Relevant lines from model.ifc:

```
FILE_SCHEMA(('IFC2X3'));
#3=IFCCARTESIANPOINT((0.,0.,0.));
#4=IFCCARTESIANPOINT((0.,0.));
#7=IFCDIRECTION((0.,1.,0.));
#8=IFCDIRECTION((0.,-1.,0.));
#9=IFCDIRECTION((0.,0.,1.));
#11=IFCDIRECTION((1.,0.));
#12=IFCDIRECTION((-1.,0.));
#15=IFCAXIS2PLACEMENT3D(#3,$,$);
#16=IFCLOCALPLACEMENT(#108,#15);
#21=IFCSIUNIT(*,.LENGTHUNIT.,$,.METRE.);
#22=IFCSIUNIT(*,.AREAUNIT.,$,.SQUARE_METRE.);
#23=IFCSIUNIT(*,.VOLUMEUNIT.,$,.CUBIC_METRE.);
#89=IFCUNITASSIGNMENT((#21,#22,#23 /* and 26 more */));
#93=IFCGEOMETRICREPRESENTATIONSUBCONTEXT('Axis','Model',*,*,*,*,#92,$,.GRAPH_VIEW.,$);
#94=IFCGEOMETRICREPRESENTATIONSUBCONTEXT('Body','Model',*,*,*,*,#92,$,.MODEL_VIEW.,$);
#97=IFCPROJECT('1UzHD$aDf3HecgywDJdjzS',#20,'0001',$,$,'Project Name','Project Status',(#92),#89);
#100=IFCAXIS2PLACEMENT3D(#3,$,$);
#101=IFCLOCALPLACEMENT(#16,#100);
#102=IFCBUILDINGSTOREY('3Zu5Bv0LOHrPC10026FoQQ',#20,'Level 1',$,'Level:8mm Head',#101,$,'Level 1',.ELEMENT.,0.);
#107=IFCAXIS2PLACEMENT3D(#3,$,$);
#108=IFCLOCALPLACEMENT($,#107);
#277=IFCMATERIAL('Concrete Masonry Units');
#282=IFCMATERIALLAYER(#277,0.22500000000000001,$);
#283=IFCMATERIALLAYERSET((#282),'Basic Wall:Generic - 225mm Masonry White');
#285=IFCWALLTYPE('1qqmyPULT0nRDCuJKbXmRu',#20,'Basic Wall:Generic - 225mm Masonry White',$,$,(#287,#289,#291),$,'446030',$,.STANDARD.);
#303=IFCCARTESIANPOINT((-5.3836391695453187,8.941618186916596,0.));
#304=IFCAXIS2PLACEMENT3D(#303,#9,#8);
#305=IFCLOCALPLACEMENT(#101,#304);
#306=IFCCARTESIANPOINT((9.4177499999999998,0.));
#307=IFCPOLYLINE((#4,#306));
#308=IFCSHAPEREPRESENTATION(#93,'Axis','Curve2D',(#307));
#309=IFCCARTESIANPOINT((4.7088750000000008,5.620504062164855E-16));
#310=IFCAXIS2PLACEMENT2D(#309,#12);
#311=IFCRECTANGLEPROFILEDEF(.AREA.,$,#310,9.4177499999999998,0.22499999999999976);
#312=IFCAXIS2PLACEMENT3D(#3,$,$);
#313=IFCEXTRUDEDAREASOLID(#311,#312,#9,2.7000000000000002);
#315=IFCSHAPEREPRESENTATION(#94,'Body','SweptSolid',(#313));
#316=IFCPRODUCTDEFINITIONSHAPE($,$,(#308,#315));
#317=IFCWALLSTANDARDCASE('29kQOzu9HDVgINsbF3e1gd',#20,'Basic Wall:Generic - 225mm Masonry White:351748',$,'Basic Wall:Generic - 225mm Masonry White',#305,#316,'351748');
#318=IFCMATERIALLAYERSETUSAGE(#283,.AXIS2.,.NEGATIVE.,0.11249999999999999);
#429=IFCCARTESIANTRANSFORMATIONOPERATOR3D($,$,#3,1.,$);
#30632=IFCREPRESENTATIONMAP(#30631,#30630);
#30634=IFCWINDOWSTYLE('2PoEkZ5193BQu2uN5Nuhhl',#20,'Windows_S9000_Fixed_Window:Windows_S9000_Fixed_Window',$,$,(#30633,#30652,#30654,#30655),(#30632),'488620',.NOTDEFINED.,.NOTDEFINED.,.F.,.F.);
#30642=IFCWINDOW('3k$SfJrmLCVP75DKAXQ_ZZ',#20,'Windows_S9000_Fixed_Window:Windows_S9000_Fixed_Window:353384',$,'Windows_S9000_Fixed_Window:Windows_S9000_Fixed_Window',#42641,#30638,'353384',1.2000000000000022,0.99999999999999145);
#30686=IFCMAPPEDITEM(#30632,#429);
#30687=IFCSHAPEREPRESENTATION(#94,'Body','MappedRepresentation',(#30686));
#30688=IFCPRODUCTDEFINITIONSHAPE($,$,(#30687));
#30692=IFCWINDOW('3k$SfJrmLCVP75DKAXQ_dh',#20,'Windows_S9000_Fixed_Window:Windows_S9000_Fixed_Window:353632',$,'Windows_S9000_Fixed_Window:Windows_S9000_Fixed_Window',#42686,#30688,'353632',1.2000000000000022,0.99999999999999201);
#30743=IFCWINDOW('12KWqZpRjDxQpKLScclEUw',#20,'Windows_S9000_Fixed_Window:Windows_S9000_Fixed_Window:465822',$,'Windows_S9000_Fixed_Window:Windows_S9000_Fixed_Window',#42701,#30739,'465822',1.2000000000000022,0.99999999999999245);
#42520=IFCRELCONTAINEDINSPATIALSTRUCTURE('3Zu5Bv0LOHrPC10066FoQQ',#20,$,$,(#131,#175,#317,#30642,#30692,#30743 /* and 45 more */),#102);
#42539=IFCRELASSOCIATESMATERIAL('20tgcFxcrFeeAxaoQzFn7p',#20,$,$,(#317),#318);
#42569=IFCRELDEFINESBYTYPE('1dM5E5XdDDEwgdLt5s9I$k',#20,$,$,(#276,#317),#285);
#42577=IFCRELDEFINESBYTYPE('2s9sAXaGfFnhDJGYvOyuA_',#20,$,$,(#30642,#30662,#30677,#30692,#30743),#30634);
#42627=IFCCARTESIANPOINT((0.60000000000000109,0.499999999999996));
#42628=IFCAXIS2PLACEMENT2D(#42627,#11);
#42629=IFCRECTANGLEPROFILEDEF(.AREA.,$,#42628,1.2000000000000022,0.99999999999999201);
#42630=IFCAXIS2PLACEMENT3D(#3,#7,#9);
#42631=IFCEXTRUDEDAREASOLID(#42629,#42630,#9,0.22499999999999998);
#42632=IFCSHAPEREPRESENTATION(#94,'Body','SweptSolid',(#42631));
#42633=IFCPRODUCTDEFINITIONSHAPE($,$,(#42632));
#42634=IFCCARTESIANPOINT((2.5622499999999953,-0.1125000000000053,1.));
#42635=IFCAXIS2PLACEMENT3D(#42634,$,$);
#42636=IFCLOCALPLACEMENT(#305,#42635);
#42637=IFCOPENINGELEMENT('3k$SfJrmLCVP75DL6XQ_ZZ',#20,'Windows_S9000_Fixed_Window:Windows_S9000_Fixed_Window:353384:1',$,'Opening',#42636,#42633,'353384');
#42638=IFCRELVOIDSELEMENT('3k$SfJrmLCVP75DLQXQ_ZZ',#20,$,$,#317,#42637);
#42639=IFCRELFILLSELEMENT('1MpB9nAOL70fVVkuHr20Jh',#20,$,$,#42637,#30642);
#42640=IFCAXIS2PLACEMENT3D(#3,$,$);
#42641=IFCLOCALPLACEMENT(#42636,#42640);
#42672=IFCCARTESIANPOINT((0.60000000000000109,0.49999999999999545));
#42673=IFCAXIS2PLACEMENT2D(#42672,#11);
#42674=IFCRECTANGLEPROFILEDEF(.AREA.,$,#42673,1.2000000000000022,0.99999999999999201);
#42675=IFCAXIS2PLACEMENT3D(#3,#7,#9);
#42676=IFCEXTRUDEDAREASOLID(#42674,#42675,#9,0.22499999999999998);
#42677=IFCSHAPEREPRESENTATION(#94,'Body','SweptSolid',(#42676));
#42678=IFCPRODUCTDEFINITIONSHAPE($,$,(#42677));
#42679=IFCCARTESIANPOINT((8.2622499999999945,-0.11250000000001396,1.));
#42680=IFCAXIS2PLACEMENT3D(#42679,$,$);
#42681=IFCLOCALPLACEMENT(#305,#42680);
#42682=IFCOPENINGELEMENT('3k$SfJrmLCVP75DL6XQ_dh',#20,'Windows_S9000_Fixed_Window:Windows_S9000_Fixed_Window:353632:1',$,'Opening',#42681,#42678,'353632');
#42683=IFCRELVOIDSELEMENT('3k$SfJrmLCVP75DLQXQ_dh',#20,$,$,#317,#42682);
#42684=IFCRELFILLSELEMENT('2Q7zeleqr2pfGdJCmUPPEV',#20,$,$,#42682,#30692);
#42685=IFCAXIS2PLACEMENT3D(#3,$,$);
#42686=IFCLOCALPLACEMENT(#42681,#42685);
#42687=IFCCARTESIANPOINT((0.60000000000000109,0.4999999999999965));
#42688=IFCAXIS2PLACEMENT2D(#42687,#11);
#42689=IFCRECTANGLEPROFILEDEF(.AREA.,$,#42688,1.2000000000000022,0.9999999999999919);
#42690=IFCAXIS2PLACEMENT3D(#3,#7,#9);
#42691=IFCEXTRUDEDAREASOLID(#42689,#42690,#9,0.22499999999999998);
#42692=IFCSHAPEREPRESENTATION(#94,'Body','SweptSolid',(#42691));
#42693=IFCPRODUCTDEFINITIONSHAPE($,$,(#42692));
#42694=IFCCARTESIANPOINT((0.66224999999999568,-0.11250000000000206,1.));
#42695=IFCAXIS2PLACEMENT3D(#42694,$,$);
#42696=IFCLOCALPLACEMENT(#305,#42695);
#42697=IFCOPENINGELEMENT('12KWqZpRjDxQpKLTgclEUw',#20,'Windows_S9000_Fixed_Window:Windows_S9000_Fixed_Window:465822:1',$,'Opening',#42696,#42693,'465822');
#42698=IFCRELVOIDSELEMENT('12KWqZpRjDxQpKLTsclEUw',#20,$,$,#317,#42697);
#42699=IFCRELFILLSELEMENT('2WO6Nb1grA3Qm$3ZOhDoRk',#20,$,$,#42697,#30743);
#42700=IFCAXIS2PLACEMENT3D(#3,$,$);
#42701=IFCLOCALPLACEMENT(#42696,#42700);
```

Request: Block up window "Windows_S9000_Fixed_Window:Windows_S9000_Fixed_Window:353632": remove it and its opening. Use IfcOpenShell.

```python
import ifcopenshell
import ifcopenshell.api.feature
import ifcopenshell.api.root
import ifcopenshell.geom
import ifcopenshell.util.shape

model = ifcopenshell.open("model.ifc")
settings = ifcopenshell.geom.settings()


def volume(element):
    """Net volume in cubic metres, openings subtracted."""
    shape = ifcopenshell.geom.create_shape(settings, element)
    return ifcopenshell.util.shape.get_volume(shape.geometry)


window = model.by_guid("3k$SfJrmLCVP75DKAXQ_dh")
opening = window.FillsVoids[0].RelatingOpeningElement
wall = opening.VoidsElements[0].RelatingBuildingElement
before = volume(wall)

ifcopenshell.api.root.remove_product(model, product=window)
ifcopenshell.api.feature.remove_feature(model, feature=opening)

after = volume(wall)

print(f"wall volume {before:.3f} -> {after:.3f} m3")

model.write("model_edited.ifc")
```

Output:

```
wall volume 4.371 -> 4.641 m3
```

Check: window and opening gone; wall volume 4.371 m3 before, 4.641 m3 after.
